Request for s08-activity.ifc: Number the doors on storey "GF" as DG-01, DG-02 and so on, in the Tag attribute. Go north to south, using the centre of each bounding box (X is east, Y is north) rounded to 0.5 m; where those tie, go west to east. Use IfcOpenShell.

First a look at what the model holds.

```python
import ifcopenshell
import ifcopenshell.util.element
import ifcopenshell.util.placement

model = ifcopenshell.open("s08-activity.ifc")
print(model.schema)
storey = next(s for s in model.by_type("IfcBuildingStorey") if s.Name == "GF")
doors = [e for e in ifcopenshell.util.element.get_decomposition(storey) if e.is_a("IfcDoor")]
for e in sorted(doors, key=lambda e: e.id()):
    origin = ifcopenshell.util.placement.get_local_placement(e.ObjectPlacement)[:3, 3]
    print(e.id(), e.Tag, e.Name, origin.round(2) + 0.0, sep=" | ")
```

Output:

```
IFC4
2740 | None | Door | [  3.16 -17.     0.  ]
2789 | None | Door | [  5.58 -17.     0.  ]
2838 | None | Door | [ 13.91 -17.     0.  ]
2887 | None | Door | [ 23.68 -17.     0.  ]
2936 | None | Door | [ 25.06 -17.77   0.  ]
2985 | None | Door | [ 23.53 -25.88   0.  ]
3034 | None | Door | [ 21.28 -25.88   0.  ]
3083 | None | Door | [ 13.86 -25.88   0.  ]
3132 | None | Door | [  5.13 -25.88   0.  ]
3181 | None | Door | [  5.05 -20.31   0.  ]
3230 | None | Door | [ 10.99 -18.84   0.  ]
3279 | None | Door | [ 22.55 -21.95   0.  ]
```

```python
import ifcopenshell
import ifcopenshell.geom
import ifcopenshell.util.element
import ifcopenshell.util.shape

model = ifcopenshell.open("s08-activity.ifc")
settings = ifcopenshell.geom.settings()
settings.set("use-world-coords", True)


def centre(element):
    shape = ifcopenshell.geom.create_shape(settings, element)
    return ifcopenshell.util.shape.get_bbox_centroid(shape.geometry)


storey = next(s for s in model.by_type("IfcBuildingStorey") if s.Name == "GF")
doors = [e for e in ifcopenshell.util.element.get_decomposition(storey) if e.is_a("IfcDoor")]

# Insertion points can sit at a corner or the storey origin, so sort by the geometry (in metres).
centres = {e: centre(e) for e in doors}
doors.sort(key=lambda e: (-round(centres[e][1] / 0.5), centres[e][0]))

for i, e in enumerate(doors, start=1):
    number = f"DG-{i:02d}"
    e.Tag = number
    print(e.id(), number)

model.write("s08-activity_edited.ifc")
```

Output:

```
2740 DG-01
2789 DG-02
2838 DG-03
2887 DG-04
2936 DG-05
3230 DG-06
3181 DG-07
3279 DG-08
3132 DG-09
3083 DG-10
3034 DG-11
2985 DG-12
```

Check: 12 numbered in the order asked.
